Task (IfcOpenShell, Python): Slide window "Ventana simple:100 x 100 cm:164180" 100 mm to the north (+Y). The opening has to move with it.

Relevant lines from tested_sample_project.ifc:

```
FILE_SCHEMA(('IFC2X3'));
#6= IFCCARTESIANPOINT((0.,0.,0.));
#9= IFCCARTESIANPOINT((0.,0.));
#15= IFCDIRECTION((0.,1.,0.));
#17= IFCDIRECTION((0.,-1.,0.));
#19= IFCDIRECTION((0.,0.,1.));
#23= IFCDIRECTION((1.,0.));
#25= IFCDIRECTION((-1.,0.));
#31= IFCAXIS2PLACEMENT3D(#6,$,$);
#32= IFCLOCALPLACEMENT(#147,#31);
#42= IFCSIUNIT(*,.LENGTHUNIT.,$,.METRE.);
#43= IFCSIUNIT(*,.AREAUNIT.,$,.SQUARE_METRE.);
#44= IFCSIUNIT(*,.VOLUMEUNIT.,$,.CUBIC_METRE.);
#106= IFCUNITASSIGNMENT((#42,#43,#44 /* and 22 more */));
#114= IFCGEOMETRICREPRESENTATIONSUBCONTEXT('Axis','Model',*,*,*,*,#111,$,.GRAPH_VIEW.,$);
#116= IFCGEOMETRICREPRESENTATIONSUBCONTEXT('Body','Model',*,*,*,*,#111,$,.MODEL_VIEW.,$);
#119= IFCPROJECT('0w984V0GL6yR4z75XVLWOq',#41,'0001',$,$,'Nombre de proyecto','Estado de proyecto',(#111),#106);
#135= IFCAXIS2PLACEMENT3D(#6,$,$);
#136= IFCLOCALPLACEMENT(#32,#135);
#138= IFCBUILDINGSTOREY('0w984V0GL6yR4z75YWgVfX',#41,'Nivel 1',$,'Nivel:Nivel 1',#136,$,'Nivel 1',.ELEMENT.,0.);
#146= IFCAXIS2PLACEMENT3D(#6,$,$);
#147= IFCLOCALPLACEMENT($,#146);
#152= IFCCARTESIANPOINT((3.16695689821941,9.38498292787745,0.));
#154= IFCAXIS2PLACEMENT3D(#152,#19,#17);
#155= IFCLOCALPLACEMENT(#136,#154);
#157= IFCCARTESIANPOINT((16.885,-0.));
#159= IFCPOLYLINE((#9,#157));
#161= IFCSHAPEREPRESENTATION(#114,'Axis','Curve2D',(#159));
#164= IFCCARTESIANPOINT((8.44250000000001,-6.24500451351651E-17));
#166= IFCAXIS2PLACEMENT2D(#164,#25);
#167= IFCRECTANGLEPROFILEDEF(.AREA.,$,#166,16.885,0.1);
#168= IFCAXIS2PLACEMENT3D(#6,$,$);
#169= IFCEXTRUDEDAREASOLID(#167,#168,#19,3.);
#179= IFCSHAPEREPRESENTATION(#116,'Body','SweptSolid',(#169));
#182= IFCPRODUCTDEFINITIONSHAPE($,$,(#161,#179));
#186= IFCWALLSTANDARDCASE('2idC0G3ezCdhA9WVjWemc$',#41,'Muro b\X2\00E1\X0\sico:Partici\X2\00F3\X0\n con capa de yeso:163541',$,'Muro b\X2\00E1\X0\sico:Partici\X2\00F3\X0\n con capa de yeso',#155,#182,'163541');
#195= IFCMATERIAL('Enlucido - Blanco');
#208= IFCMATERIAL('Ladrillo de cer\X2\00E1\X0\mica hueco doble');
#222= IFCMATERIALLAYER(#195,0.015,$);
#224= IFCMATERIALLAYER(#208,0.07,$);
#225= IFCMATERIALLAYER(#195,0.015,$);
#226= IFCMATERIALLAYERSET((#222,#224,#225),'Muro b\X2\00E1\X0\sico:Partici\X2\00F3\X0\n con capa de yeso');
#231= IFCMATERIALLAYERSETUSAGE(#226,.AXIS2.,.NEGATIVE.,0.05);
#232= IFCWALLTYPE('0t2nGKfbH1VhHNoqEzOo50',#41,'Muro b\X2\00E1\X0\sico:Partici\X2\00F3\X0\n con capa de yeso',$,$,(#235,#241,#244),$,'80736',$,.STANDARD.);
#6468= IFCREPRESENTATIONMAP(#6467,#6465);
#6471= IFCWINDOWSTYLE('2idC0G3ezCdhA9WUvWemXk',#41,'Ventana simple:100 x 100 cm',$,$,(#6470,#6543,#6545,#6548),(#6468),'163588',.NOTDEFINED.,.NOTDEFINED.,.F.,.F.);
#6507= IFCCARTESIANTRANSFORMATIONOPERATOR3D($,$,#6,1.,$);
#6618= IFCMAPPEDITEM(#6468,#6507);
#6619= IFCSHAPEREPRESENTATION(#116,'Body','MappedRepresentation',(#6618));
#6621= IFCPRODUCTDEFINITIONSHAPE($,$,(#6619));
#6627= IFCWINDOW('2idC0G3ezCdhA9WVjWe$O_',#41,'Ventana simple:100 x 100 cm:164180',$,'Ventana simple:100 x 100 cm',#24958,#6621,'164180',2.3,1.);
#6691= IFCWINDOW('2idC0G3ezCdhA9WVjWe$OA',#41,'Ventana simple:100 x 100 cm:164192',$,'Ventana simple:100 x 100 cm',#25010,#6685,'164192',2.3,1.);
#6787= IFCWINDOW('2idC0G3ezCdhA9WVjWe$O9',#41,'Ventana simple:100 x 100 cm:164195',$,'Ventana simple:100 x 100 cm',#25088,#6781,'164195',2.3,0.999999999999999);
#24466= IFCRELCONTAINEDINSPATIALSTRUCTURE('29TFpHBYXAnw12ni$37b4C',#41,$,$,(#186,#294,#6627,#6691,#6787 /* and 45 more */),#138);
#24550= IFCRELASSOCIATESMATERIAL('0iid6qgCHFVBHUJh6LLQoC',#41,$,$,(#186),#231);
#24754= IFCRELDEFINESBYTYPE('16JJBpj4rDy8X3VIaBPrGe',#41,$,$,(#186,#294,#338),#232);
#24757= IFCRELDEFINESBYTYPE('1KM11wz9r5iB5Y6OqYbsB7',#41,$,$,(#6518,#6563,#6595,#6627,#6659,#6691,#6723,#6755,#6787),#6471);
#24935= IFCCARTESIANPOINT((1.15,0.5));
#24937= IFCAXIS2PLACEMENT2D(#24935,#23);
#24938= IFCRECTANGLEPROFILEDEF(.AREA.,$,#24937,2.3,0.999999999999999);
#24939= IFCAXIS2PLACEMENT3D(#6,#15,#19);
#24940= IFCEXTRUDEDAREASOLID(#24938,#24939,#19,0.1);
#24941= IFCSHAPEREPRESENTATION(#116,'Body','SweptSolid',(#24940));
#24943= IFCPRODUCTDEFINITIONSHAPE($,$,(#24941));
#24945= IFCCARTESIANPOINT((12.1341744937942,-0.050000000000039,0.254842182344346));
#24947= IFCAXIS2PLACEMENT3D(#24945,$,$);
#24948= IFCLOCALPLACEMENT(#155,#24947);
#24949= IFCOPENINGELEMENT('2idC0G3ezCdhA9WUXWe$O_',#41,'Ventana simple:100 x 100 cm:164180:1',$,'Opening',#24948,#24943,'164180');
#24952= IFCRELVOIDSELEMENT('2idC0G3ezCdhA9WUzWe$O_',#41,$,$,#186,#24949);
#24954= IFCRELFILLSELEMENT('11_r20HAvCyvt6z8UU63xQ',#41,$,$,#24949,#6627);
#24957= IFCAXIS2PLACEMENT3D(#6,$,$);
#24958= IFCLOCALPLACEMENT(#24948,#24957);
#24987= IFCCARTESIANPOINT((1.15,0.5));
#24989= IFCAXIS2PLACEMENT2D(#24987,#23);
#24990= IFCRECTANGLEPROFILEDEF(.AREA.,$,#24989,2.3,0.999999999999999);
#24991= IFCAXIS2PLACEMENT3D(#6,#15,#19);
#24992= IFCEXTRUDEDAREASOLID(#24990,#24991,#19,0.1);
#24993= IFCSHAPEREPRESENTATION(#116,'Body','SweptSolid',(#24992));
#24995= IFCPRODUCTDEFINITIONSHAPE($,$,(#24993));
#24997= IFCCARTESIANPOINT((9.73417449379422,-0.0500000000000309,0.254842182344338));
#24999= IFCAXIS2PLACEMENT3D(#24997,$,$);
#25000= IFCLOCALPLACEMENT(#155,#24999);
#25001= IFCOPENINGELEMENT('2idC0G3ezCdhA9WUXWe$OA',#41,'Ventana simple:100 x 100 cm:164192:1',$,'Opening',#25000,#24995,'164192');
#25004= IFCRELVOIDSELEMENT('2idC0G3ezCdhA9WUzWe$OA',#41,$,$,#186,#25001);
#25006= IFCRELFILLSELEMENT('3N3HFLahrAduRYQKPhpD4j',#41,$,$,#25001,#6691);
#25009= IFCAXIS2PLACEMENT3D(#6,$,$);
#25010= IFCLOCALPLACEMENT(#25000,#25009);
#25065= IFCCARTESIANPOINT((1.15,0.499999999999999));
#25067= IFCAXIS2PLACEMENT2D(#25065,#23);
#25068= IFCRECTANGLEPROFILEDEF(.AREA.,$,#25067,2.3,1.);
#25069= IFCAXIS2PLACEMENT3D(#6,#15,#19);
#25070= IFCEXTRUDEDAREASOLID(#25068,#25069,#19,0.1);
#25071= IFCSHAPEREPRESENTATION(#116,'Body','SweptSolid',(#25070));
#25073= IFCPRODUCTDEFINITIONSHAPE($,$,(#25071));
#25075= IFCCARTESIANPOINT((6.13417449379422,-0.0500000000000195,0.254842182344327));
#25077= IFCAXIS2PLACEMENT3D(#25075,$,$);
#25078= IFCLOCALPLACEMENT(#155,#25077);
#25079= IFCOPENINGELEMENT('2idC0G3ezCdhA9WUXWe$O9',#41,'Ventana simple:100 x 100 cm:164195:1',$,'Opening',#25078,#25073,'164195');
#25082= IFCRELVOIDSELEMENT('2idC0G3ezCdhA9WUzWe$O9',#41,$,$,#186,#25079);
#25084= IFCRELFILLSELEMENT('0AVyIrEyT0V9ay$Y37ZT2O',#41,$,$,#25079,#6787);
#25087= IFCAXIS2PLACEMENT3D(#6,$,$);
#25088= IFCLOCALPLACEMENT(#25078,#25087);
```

```python
import ifcopenshell
import ifcopenshell.api.geometry
import ifcopenshell.util.placement
import ifcopenshell.util.unit

model = ifcopenshell.open("tested_sample_project.ifc")
unit_scale = ifcopenshell.util.unit.calculate_unit_scale(model)

window = model.by_guid("2idC0G3ezCdhA9WVjWe$O_")
opening = window.FillsVoids[0].RelatingOpeningElement
wall = opening.VoidsElements[0].RelatingBuildingElement

wall_matrix = ifcopenshell.util.placement.get_local_placement(wall.ObjectPlacement)
shift = wall_matrix[:3, 0] * -0.1 / unit_scale
before = ifcopenshell.util.placement.get_local_placement(window.ObjectPlacement)[:3, 3].copy()

# The window is placed relative to its opening, so it follows when the opening moves.
matrix = ifcopenshell.util.placement.get_local_placement(opening.ObjectPlacement)
matrix[:3, 3] += shift
ifcopenshell.api.geometry.edit_object_placement(
    model, product=opening, matrix=matrix, is_si=False, should_transform_children=True
)

after = ifcopenshell.util.placement.get_local_placement(window.ObjectPlacement)[:3, 3]
print("window moved by", (after - before).round(3) + 0.0)

model.write("tested_sample_project_v2.ifc")
```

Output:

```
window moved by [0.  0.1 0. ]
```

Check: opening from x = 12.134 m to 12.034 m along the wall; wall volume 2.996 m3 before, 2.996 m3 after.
